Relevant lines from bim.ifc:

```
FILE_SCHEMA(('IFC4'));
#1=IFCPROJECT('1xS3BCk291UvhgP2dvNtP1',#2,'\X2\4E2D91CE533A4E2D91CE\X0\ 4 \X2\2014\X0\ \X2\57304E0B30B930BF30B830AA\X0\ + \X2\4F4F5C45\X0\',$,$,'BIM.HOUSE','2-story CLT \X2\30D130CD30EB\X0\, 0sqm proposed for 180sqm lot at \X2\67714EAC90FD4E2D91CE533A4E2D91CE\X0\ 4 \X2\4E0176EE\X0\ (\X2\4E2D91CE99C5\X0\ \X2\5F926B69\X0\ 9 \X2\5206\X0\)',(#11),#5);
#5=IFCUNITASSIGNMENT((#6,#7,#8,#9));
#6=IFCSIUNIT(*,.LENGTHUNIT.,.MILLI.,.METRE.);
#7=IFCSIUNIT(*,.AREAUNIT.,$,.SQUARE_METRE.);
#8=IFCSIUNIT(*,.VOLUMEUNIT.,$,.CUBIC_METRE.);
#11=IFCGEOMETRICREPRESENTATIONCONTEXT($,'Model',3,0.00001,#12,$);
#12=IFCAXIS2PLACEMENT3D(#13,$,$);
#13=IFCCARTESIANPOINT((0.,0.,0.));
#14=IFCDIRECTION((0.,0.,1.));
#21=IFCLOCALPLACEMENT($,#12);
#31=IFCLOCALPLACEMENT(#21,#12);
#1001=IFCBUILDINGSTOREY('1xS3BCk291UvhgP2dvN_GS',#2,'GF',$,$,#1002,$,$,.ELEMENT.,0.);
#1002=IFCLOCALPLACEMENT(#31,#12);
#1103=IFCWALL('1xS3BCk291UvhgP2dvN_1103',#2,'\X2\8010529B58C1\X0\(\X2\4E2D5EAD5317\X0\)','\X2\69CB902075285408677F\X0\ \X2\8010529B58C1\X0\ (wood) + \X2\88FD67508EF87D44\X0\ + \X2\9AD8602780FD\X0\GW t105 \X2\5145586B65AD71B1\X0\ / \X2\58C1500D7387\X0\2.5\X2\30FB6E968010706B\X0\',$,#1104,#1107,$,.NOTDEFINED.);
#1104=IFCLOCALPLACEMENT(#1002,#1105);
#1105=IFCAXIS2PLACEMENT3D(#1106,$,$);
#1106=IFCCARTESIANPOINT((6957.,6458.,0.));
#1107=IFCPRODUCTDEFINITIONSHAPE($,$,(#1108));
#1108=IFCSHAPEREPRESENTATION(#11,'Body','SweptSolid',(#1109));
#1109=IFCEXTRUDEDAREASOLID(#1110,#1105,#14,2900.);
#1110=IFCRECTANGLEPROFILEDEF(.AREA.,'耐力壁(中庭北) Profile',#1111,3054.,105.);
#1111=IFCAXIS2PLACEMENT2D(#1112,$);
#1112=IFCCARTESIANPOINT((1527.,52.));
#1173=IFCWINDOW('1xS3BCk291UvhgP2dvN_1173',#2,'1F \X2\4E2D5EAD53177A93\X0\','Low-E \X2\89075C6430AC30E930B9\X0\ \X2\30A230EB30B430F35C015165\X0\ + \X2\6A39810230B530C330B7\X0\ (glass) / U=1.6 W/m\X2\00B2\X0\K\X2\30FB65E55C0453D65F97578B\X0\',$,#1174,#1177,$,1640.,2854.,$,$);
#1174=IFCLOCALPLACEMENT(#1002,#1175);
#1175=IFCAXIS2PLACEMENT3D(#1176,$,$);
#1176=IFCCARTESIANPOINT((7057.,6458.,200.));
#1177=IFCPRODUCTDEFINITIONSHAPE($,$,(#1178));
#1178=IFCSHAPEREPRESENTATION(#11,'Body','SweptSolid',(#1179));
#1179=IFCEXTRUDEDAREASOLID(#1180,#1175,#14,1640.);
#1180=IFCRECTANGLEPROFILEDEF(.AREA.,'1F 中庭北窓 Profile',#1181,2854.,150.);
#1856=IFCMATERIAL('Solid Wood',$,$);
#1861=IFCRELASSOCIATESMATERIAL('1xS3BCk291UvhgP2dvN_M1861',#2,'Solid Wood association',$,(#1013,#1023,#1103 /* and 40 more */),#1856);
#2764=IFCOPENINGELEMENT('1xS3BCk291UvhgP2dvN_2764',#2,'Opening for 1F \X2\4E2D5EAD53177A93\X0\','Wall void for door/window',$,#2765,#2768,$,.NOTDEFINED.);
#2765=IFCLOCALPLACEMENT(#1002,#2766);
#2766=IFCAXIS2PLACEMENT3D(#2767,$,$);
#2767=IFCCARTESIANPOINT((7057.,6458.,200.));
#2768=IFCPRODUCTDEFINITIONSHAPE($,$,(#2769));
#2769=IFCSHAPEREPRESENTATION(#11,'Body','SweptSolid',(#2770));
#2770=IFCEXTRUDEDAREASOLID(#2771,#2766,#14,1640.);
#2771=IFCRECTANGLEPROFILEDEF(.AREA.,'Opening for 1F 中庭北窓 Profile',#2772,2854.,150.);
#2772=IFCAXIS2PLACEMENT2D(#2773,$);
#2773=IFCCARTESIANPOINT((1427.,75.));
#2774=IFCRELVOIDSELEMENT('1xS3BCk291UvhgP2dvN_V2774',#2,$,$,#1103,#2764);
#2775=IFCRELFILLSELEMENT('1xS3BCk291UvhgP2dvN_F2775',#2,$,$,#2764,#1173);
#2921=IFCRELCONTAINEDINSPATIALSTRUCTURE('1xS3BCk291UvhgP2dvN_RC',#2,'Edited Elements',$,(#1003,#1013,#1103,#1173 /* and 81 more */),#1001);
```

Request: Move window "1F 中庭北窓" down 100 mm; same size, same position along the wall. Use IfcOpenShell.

```python
import numpy as np
import ifcopenshell
import ifcopenshell.api.geometry
import ifcopenshell.util.placement
import ifcopenshell.util.unit

model = ifcopenshell.open("bim.ifc")
unit_scale = ifcopenshell.util.unit.calculate_unit_scale(model)

window = model.by_id(1173)
opening = window.FillsVoids[0].RelatingOpeningElement
dz = -0.1 / unit_scale

shift = np.array([0.0, 0.0, dz])
# The window is not placed relative to its opening, so move both.
for product in (opening, window):
    matrix = ifcopenshell.util.placement.get_local_placement(product.ObjectPlacement)
    matrix[:3, 3] += shift
    ifcopenshell.api.geometry.edit_object_placement(model, product=product, matrix=matrix, is_si=False)

print(f"moved by {dz * unit_scale:+.3f} m")

model.write("bim_edited.ifc")
```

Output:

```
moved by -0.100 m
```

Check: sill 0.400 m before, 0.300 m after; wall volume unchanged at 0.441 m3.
